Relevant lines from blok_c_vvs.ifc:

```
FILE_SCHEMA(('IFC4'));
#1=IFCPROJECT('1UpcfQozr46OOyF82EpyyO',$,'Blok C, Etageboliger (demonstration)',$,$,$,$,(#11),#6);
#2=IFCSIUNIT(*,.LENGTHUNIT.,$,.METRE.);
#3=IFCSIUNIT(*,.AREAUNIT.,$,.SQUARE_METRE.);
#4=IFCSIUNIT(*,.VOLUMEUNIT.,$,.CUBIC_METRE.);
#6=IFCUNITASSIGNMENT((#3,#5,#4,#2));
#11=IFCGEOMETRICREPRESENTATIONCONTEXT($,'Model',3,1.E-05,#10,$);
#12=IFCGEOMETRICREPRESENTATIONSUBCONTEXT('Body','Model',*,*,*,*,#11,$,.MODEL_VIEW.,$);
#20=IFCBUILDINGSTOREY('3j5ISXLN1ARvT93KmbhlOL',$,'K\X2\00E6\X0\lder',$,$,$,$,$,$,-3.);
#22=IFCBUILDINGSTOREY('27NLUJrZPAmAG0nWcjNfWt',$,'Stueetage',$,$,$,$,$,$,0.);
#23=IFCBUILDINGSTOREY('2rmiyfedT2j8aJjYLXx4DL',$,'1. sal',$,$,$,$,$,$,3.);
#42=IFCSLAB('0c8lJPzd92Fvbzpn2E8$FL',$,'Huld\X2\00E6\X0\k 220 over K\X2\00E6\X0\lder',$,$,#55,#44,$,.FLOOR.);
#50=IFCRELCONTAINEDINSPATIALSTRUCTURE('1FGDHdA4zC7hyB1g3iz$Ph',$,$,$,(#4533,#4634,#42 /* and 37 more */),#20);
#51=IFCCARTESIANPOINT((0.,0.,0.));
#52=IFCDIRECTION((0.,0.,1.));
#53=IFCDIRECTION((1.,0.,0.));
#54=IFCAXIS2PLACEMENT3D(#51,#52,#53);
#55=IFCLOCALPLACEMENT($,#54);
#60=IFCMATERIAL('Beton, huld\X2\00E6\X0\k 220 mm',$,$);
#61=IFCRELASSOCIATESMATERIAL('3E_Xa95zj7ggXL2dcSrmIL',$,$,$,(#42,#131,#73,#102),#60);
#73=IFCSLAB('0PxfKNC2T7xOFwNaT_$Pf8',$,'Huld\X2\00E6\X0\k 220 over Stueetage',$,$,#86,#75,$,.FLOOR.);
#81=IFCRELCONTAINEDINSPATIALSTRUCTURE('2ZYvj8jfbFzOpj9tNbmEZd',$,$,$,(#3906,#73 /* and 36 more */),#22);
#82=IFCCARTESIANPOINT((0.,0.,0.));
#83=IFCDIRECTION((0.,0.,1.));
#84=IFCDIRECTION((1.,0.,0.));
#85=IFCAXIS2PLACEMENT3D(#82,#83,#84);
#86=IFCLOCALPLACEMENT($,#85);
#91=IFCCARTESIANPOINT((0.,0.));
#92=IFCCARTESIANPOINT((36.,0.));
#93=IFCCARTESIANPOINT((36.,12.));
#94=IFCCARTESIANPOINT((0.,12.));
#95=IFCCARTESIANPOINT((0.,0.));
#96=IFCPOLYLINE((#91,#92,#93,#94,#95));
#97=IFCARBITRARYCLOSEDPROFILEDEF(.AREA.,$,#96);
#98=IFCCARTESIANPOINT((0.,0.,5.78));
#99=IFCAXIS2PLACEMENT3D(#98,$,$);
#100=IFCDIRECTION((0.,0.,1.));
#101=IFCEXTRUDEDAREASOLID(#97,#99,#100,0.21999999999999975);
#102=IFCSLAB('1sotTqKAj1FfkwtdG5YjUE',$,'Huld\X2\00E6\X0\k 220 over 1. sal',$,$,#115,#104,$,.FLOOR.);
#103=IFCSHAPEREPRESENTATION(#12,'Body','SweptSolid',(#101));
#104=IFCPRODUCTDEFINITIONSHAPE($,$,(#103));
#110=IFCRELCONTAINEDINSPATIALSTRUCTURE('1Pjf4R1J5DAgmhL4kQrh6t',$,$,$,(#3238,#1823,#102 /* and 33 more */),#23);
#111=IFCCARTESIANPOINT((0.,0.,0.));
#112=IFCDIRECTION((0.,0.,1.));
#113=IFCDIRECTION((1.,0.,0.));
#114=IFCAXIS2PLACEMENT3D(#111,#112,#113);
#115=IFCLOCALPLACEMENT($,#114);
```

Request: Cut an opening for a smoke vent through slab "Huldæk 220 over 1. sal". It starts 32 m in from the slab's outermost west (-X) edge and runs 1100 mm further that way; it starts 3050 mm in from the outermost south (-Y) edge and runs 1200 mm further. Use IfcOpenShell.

```python
import numpy as np
import ifcopenshell
import ifcopenshell.api.feature
import ifcopenshell.api.geometry
import ifcopenshell.api.root
import ifcopenshell.geom
import ifcopenshell.util.placement
import ifcopenshell.util.representation
import ifcopenshell.util.shape
import ifcopenshell.util.unit

model = ifcopenshell.open("blok_c_vvs.ifc")
unit_scale = ifcopenshell.util.unit.calculate_unit_scale(model)
settings = ifcopenshell.geom.settings()


def volume(element):
    """Net volume in cubic metres, openings subtracted."""
    shape = ifcopenshell.geom.create_shape(settings, element)
    return ifcopenshell.util.shape.get_volume(shape.geometry)


slab = model.by_id(102)
before = volume(slab)

# Extent in the slab's own axes, in metres. The edges named are its -X and -Y sides.
slab_shape = ifcopenshell.geom.create_shape(settings, slab)
vertices = ifcopenshell.util.shape.get_vertices(slab_shape.geometry)
x_min, y_min, bottom = vertices.min(axis=0)
top = vertices[:, 2].max()

opening = ifcopenshell.api.root.create_entity(model, ifc_class="IfcOpeningElement", name="Smoke vent opening", predefined_type="OPENING")
context = ifcopenshell.util.representation.get_context(model, "Model", "Body", "MODEL_VIEW")
width, depth = 1.1, 1.2
outline = [(0.0, 0.0), (width, 0.0), (width, depth), (0.0, depth), (0.0, 0.0)]
# Overshoot both faces by 50 mm so the cut is clean.
shape = ifcopenshell.api.geometry.add_slab_representation(
    model, context=context, depth=top - bottom + 0.1, polyline=outline
)
ifcopenshell.api.geometry.assign_representation(model, product=opening, representation=shape)

matrix = ifcopenshell.util.placement.get_local_placement(slab.ObjectPlacement)
matrix[:, 3] = matrix @ np.append(np.array([x_min + 32, y_min + 3.05, bottom - 0.05]) / unit_scale, 1.0)
ifcopenshell.api.geometry.edit_object_placement(model, product=opening, matrix=matrix, is_si=False)
ifcopenshell.api.feature.add_feature(model, feature=opening, element=slab)

after = volume(slab)

print(f"slab volume {before:.3f} -> {after:.3f} m3")

model.write("blok_c_vvs_edited.ifc")
```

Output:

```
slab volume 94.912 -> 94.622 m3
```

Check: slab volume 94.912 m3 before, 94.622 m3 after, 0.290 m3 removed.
